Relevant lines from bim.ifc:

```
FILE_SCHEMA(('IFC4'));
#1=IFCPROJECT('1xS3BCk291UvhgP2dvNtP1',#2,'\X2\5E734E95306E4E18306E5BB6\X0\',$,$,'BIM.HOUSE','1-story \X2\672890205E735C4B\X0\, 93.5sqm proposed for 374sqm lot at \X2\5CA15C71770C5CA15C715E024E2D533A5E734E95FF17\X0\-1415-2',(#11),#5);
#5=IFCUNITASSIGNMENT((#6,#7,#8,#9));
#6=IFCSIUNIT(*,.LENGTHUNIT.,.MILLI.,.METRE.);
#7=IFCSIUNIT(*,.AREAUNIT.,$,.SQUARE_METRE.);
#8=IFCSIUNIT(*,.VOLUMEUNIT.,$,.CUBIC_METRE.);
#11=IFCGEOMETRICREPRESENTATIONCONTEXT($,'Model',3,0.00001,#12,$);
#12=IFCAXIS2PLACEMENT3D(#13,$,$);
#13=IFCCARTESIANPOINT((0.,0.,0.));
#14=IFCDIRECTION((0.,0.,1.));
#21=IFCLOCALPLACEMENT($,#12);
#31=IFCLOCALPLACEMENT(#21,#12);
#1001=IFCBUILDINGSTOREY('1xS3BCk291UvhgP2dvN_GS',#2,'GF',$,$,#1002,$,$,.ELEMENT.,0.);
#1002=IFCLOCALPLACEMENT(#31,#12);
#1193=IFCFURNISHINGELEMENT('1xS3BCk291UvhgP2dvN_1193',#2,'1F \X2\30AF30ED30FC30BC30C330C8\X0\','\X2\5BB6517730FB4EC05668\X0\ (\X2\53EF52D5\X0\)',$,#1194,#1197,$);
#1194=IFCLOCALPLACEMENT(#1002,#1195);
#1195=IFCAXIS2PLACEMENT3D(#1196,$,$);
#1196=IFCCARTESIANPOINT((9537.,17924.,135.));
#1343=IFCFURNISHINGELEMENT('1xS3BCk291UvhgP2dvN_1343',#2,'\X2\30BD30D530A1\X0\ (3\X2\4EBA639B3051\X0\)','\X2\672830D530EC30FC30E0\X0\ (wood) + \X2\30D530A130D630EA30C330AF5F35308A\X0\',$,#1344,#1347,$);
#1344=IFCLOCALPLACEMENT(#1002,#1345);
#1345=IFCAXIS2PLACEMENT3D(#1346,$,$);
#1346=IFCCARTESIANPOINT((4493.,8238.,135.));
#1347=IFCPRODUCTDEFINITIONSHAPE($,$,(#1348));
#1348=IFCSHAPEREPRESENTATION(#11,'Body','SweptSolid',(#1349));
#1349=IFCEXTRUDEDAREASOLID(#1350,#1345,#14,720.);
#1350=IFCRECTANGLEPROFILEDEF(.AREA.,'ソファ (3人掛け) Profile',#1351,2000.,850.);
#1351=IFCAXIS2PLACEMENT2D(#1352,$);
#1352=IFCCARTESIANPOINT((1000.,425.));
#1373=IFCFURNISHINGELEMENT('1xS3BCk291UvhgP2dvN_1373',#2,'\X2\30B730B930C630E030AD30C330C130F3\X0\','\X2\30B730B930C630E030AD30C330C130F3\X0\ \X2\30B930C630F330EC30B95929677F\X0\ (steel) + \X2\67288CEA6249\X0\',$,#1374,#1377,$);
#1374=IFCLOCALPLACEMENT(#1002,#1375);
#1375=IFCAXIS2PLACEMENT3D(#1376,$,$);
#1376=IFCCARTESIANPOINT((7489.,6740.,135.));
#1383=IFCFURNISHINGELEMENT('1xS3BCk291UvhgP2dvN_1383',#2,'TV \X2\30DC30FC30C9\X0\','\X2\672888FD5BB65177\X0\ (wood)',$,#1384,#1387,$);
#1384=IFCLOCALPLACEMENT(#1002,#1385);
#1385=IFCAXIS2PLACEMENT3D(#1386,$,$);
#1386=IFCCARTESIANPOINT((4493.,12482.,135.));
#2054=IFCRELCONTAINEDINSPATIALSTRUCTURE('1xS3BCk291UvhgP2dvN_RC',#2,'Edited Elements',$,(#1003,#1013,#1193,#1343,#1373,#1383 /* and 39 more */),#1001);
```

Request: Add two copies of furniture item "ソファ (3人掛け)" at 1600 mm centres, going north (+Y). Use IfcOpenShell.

```python
import numpy as np
import ifcopenshell
import ifcopenshell.api.geometry
import ifcopenshell.api.root
import ifcopenshell.util.element
import ifcopenshell.util.placement
import ifcopenshell.util.unit

model = ifcopenshell.open("bim.ifc")
unit_scale = ifcopenshell.util.unit.calculate_unit_scale(model)


def reuse_history(source, copy):
    """copy_class also copies each property set's owner history, people and application; keep the originals."""
    for rel in copy.IsDefinedBy:
        if rel.is_a("IfcRelDefinesByProperties") and (history := rel.RelatingPropertyDefinition.OwnerHistory):
            rel.RelatingPropertyDefinition.OwnerHistory = source.OwnerHistory
            ifcopenshell.util.element.remove_deep2(model, history)


source = model.by_id(1343)
base = ifcopenshell.util.placement.get_local_placement(source.ObjectPlacement)
step = np.array([0.0, 1.0, 0.0]) * 1.6 / unit_scale

for i in range(1, 3):
    copy = ifcopenshell.api.root.copy_class(model, product=source)
    copy.Representation = ifcopenshell.util.element.copy_deep(
        model, source.Representation, exclude=["IfcGeometricRepresentationContext", "IfcRepresentationMap"]
    )
    reuse_history(source, copy)
    matrix = base.copy()
    matrix[:3, 3] += i * step
    print("added at", matrix[:3, 3].round(3) + 0.0)
    ifcopenshell.api.geometry.edit_object_placement(model, product=copy, matrix=matrix, is_si=False)

model.write("bim_rev.ifc")
```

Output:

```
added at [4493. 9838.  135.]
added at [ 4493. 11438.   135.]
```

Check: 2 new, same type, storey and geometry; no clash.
